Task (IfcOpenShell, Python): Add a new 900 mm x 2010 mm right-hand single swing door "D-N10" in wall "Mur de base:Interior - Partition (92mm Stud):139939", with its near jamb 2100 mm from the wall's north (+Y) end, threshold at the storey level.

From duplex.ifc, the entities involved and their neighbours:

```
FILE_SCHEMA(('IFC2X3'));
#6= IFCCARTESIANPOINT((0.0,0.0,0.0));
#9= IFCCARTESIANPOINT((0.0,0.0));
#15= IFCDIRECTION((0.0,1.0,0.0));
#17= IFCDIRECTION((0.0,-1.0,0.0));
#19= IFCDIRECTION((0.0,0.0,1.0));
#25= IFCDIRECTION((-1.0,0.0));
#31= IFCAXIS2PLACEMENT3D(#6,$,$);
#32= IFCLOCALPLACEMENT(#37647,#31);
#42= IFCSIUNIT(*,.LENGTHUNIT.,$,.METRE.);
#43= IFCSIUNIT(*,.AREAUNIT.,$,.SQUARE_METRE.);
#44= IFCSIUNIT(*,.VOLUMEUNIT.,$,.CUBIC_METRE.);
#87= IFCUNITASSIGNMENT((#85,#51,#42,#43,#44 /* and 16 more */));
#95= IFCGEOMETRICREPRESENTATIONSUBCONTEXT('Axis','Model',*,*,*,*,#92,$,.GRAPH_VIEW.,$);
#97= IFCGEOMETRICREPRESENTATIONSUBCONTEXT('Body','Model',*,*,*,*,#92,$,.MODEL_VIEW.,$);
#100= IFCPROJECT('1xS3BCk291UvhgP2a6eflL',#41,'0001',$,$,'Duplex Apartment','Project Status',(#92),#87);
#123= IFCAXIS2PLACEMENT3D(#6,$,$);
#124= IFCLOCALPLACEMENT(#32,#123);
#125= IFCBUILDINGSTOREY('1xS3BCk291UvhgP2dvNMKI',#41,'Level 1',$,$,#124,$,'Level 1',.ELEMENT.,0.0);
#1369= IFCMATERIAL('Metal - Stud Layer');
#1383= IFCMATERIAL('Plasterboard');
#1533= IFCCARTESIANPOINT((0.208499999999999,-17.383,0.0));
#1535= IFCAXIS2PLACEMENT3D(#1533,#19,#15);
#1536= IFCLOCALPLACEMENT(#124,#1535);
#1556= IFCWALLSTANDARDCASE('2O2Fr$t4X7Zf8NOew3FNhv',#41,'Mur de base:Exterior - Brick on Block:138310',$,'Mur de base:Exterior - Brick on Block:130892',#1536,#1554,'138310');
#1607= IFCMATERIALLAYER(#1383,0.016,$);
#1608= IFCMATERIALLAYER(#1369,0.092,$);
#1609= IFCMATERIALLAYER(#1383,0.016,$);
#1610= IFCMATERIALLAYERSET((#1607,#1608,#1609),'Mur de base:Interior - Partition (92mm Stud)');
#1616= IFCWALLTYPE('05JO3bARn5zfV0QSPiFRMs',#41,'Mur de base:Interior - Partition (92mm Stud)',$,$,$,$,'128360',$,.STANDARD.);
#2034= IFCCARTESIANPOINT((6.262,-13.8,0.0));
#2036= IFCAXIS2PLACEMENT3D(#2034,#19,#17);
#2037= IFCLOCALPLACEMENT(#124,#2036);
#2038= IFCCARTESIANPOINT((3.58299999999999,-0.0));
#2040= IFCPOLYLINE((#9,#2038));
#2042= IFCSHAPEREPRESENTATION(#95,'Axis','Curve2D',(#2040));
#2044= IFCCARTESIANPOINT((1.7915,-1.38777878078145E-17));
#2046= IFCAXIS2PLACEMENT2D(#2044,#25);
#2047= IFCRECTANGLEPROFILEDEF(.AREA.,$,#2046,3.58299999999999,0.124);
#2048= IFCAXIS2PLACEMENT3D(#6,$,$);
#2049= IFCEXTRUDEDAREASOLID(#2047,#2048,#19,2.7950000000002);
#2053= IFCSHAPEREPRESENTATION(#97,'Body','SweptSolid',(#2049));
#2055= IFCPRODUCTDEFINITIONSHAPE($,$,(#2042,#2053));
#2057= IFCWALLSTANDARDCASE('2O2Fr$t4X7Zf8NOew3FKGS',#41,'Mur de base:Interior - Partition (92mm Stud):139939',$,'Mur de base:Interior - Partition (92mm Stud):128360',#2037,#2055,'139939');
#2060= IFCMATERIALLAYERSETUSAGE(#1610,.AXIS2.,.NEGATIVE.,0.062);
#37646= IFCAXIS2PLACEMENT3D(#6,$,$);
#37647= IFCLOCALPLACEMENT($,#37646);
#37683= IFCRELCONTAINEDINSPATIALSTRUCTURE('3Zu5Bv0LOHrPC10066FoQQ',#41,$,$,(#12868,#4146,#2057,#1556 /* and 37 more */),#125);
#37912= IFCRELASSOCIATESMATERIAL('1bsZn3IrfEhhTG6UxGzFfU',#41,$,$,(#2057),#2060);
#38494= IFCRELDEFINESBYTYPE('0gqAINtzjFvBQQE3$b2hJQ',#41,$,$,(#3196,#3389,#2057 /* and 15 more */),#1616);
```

```python
import numpy as np
import ifcopenshell
import ifcopenshell.api.feature
import ifcopenshell.api.geometry
import ifcopenshell.api.root
import ifcopenshell.api.spatial
import ifcopenshell.api.type
import ifcopenshell.geom
import ifcopenshell.util.element
import ifcopenshell.util.placement
import ifcopenshell.util.representation
import ifcopenshell.util.shape
import ifcopenshell.util.unit

model = ifcopenshell.open("duplex.ifc")
unit_scale = ifcopenshell.util.unit.calculate_unit_scale(model)
settings = ifcopenshell.geom.settings()


def volume(element):
    """Net volume in cubic metres, openings subtracted."""
    shape = ifcopenshell.geom.create_shape(settings, element)
    return ifcopenshell.util.shape.get_volume(shape.geometry)


wall = model.by_guid("2O2Fr$t4X7Zf8NOew3FKGS")
storey = ifcopenshell.util.element.get_container(wall, ifc_class="IfcBuildingStorey")
context = ifcopenshell.util.representation.get_context(model, "Model", "Body", "MODEL_VIEW")
before = volume(wall)

width, height, from_end, sill = 0.9, 2.01, 2.1, 0.0  # metres

# The wall runs along its own X axis, and the end named is its -X end.
wall_shape = ifcopenshell.geom.create_shape(settings, wall)
x, y, z = ifcopenshell.util.shape.get_vertices(wall_shape.geometry).T
start = x.min() + from_end
face, thickness = float(y.min()), float(y.max() - y.min())
wall_matrix = ifcopenshell.util.placement.get_local_placement(wall.ObjectPlacement)
level = ifcopenshell.util.placement.get_local_placement(storey.ObjectPlacement)[2, 3]


def in_wall(x, y):
    """Placement at x, y metres in the wall's axes, at sill height."""
    matrix = wall_matrix.copy()
    matrix[:, 3] = wall_matrix @ np.array([x / unit_scale, y / unit_scale, 0.0, 1.0])
    matrix[2, 3] = level + sill / unit_scale
    return matrix


# Opening: a box that overshoots both wall faces by 50 mm.
opening = ifcopenshell.api.root.create_entity(model, ifc_class="IfcOpeningElement")
box = ifcopenshell.api.geometry.add_wall_representation(
    model, context=context, length=width, height=height, thickness=thickness + 0.1
)
ifcopenshell.api.geometry.assign_representation(model, product=opening, representation=box)
ifcopenshell.api.geometry.edit_object_placement(model, product=opening, matrix=in_wall(start, face - 0.05), is_si=False)
ifcopenshell.api.feature.add_feature(model, feature=opening, element=wall)

door = ifcopenshell.api.root.create_entity(model, ifc_class="IfcDoor", name="D-N10")
door.OverallWidth, door.OverallHeight = width / unit_scale, height / unit_scale
body = ifcopenshell.api.geometry.add_door_representation(
    model,
    context=context,
    overall_width=door.OverallWidth,
    overall_height=door.OverallHeight,
    operation_type="SINGLE_SWING_RIGHT",
    lining_properties={"LiningDepth": thickness / unit_scale, "ThresholdDepth": thickness / unit_scale},
)
ifcopenshell.api.geometry.assign_representation(model, product=door, representation=body)
ifcopenshell.api.spatial.assign_container(model, products=[door], relating_structure=storey)
fills = ifcopenshell.api.feature.add_filling(model, opening=opening, element=door)
fills.OwnerHistory = door.OwnerHistory  # required in IFC2X3

# IFC2X3 keeps the operation on the door style.
style = ifcopenshell.api.root.create_entity(model, ifc_class="IfcDoorStyle", name="D-N10")
style.OperationType, style.ConstructionType = "SINGLE_SWING_RIGHT", "NOTDEFINED"
style.ParameterTakesPrecedence = style.Sizeable = False
ifcopenshell.api.type.assign_type(model, related_objects=[door], relating_type=style)

# The lining spans the wall, so the door starts at the wall face.
ifcopenshell.api.geometry.edit_object_placement(model, product=door, matrix=in_wall(start, face), is_si=False)

after = volume(wall)

print(f"wall volume {before:.3f} -> {after:.3f} m3")

model.write("duplex-out.ifc")
```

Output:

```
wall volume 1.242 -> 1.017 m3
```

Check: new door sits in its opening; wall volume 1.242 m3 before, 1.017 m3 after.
